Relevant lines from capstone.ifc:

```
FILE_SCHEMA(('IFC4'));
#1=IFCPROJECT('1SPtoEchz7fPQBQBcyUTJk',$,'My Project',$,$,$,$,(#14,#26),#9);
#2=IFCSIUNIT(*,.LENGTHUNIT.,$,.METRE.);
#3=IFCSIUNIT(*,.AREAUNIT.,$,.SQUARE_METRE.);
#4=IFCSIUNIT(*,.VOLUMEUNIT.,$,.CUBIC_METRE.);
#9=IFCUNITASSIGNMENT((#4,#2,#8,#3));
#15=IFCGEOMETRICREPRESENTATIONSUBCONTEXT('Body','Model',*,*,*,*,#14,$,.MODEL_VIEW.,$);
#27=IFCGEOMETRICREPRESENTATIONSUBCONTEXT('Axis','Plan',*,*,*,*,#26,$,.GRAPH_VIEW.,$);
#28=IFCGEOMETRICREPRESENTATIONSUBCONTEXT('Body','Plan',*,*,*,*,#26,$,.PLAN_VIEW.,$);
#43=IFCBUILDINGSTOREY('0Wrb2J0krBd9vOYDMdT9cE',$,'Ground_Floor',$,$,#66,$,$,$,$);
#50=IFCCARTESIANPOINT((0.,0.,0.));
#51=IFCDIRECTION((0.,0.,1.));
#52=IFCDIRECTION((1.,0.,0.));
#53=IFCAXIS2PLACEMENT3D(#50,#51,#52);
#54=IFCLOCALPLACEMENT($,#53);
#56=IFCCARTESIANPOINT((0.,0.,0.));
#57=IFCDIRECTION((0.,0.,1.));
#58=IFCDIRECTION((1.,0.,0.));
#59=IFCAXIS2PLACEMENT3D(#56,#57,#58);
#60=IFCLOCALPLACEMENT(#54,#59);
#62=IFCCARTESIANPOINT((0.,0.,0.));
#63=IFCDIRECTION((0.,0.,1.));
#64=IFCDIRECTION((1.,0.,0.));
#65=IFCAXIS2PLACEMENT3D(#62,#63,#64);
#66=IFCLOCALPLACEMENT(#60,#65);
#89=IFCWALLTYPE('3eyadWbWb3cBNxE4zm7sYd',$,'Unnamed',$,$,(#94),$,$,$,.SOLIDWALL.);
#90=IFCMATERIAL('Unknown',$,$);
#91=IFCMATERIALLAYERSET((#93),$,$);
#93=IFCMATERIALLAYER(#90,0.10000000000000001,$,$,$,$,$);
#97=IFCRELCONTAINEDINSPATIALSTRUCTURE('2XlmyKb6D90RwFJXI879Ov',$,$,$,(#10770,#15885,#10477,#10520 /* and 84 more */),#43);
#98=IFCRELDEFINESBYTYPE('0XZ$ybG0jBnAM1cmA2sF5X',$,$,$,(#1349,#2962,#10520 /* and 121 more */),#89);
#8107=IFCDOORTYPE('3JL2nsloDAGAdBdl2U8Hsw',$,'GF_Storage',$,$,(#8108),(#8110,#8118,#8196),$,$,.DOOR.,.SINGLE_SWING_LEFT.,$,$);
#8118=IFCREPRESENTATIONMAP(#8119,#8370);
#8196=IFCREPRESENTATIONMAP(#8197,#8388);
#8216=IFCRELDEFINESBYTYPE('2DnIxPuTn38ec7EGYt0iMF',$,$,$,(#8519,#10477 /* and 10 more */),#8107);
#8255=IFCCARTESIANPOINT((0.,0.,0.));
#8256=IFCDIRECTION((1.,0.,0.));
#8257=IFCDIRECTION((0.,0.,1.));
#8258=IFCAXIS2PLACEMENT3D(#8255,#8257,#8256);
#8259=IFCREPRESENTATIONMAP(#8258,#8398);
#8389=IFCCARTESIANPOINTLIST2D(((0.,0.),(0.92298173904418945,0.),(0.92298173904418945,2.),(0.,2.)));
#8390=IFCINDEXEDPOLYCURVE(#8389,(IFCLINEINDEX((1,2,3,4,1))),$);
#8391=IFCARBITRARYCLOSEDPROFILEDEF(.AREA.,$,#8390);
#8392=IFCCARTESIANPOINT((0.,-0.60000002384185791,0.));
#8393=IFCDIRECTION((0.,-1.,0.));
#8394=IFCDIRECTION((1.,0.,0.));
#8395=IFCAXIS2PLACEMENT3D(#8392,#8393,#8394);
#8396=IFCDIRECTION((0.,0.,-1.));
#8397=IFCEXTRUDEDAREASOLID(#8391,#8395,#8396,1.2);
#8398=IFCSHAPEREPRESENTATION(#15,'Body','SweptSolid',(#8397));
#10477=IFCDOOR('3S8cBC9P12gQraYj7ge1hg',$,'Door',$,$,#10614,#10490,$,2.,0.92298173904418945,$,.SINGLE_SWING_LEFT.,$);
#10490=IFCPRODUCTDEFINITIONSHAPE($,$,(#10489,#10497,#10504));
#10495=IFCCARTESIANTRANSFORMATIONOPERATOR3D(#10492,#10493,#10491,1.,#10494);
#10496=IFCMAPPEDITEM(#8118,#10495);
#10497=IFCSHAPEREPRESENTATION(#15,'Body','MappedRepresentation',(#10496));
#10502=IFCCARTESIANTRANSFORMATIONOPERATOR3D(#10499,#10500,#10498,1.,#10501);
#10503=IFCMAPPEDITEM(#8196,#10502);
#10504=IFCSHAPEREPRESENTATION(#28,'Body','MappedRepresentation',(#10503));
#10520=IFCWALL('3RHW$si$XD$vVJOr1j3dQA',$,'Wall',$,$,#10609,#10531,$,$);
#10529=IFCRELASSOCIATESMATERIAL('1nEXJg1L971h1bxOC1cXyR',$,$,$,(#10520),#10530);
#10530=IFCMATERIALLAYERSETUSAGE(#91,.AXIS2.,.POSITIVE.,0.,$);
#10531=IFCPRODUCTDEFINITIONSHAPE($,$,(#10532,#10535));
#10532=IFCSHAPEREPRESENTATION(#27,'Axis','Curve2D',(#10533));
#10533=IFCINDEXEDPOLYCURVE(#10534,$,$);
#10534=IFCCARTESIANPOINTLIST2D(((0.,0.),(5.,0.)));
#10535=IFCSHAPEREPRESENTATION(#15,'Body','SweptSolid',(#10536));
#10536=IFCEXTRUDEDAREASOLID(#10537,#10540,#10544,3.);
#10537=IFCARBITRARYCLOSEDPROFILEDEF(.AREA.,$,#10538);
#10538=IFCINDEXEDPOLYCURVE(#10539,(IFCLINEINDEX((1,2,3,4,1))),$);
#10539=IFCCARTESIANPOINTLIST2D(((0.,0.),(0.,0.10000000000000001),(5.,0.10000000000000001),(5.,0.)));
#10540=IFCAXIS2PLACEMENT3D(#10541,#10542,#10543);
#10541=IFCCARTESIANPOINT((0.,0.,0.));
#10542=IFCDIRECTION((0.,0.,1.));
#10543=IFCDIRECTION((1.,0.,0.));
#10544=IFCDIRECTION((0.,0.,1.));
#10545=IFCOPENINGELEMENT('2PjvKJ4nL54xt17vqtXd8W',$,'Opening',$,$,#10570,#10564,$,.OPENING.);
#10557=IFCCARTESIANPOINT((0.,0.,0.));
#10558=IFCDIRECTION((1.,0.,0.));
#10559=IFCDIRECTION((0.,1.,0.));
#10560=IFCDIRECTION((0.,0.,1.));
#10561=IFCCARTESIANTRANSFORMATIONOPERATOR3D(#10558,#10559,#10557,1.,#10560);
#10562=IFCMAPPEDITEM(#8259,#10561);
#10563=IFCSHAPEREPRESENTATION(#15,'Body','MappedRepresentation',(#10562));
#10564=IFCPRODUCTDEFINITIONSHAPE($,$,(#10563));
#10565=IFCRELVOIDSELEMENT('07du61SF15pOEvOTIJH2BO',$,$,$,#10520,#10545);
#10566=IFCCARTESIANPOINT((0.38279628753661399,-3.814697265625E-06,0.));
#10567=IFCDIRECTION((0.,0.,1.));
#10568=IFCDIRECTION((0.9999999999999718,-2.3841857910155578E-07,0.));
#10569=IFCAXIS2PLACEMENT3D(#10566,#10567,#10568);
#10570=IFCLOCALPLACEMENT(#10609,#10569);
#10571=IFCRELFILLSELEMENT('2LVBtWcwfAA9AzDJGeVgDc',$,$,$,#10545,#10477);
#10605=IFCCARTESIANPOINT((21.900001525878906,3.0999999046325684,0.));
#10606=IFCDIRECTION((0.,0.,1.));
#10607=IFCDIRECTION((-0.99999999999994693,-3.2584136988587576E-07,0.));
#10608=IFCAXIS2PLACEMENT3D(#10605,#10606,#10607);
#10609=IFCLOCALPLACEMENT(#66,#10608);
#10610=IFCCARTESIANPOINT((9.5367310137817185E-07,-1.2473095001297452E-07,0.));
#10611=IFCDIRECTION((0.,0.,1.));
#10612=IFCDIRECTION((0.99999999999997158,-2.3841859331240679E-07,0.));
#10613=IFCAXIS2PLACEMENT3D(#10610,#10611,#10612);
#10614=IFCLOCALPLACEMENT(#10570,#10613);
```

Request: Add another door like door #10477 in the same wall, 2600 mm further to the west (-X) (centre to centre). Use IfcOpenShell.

```python
import ifcopenshell
import ifcopenshell.api.feature
import ifcopenshell.api.geometry
import ifcopenshell.api.root
import ifcopenshell.geom
import ifcopenshell.util.element
import ifcopenshell.util.placement
import ifcopenshell.util.shape

model = ifcopenshell.open("capstone.ifc")
settings = ifcopenshell.geom.settings()


def volume(element):
    """Net volume in cubic metres, openings subtracted."""
    shape = ifcopenshell.geom.create_shape(settings, element)
    return ifcopenshell.util.shape.get_volume(shape.geometry)


door = model.by_id(10477)
opening = door.FillsVoids[0].RelatingOpeningElement
wall = opening.VoidsElements[0].RelatingBuildingElement
before = volume(wall)
shift = ifcopenshell.util.placement.get_local_placement(wall.ObjectPlacement)[:3, 0] * 2.6

# copy_class copies the void relationship, type, container and properties, but no geometry.
new_opening = ifcopenshell.api.root.copy_class(model, product=opening)
new_opening.Representation = ifcopenshell.util.element.copy_deep(
    model, opening.Representation, exclude=["IfcGeometricRepresentationContext", "IfcRepresentationMap"]
)
new_door = ifcopenshell.api.root.copy_class(model, product=door)
new_door.Representation = ifcopenshell.util.element.copy_deep(
    model, door.Representation, exclude=["IfcGeometricRepresentationContext", "IfcRepresentationMap"]
)
ifcopenshell.api.feature.add_filling(model, opening=new_opening, element=new_door)

for old, new in ((opening, new_opening), (door, new_door)):
    matrix = ifcopenshell.util.placement.get_local_placement(old.ObjectPlacement)
    matrix[:3, 3] += shift
    ifcopenshell.api.geometry.edit_object_placement(model, product=new, matrix=matrix, is_si=False)

after = volume(wall)

print(f"wall volume {before:.3f} -> {after:.3f} m3")

model.write("capstone_rev.ifc")
```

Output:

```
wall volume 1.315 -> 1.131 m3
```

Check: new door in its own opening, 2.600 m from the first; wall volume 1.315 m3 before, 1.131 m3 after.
